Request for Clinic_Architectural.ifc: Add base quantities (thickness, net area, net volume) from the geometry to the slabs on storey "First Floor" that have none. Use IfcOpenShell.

First a look at what the model holds.

```python
import ifcopenshell
import ifcopenshell.util.element
import ifcopenshell.util.unit

model = ifcopenshell.open("Clinic_Architectural.ifc")
print(model.schema)
for unit_type in ("LENGTHUNIT", "AREAUNIT", "VOLUMEUNIT"):
    print(unit_type, ifcopenshell.util.unit.calculate_unit_scale(model, unit_type))
storey = next(s for s in model.by_type("IfcBuildingStorey") if s.Name == "First Floor")
slabs = [e for e in ifcopenshell.util.element.get_decomposition(storey) if e.is_a("IfcSlab")]
for e in sorted(slabs, key=lambda e: e.id()):
    print(e.id(), e.is_a(), e.Name, list(ifcopenshell.util.element.get_psets(e, qtos_only=True)), sep=" | ")
```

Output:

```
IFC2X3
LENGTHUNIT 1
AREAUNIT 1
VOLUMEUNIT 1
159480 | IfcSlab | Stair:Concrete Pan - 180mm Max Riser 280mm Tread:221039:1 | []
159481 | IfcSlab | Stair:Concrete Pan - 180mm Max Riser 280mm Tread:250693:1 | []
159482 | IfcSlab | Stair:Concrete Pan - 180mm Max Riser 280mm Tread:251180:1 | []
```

```python
import ifcopenshell
import ifcopenshell.api.pset
import ifcopenshell.geom
import ifcopenshell.util.element
import ifcopenshell.util.shape
import ifcopenshell.util.unit

model = ifcopenshell.open("Clinic_Architectural.ifc")
unit_scale = ifcopenshell.util.unit.calculate_unit_scale(model)
area_scale = ifcopenshell.util.unit.calculate_unit_scale(model, "AREAUNIT")
volume_scale = ifcopenshell.util.unit.calculate_unit_scale(model, "VOLUMEUNIT")
settings = ifcopenshell.geom.settings()

storey = next(s for s in model.by_type("IfcBuildingStorey") if s.Name == "First Floor")
slabs = [e for e in ifcopenshell.util.element.get_decomposition(storey) if e.is_a("IfcSlab")]

for e in sorted(slabs, key=lambda e: e.id()):
    if ifcopenshell.util.element.get_psets(e, qtos_only=True, should_inherit=False):
        continue
    # Geometry comes back in metres, in the element's own axes.
    shape = ifcopenshell.geom.create_shape(settings, e)
    values = {
        "Width": ifcopenshell.util.shape.get_z(shape.geometry) / unit_scale,
        "NetArea": ifcopenshell.util.shape.get_footprint_area(shape.geometry) / area_scale,
        "NetVolume": ifcopenshell.util.shape.get_volume(shape.geometry) / volume_scale,
    }
    qto = ifcopenshell.api.pset.add_qto(model, product=e, name="BaseQuantities")
    ifcopenshell.api.pset.edit_qto(model, qto=qto, properties=values)
    print(e.id(), {k: round(v, 3) for k, v in values.items()})

model.write("Clinic_Architectural-out.ifc")
```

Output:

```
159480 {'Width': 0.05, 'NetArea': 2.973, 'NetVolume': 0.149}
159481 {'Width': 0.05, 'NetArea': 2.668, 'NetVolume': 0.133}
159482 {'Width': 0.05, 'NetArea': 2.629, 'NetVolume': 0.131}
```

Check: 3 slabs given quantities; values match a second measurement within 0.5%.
